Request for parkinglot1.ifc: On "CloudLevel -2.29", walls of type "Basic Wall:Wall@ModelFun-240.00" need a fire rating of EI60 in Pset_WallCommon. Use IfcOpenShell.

First a look at what the model holds.

```python
import ifcopenshell
import ifcopenshell.util.element

model = ifcopenshell.open("parkinglot1.ifc")
print(model.schema)
storey = next(s for s in model.by_type("IfcBuildingStorey") if s.Name == "CloudLevel -2.29")
walls = [e for e in ifcopenshell.util.element.get_decomposition(storey) if e.is_a("IfcWall")]
seen = {}
for e in walls:
    element_type = ifcopenshell.util.element.get_type(e)
    key = (element_type.Name if element_type != e and element_type else None, ifcopenshell.util.element.get_pset(e, "Pset_WallCommon", "FireRating"))
    seen[key] = seen.get(key, 0) + 1
for (name, value), count in sorted(seen.items(), key=str):
    print(count, "x", name, "|", value)
```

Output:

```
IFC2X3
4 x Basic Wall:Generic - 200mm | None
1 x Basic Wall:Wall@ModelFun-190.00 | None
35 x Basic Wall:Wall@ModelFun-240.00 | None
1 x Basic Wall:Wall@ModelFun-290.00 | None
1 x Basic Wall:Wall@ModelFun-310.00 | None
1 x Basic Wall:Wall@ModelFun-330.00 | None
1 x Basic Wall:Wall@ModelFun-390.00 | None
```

```python
import ifcopenshell
import ifcopenshell.api.pset
import ifcopenshell.util.element

model = ifcopenshell.open("parkinglot1.ifc")

storey = next(s for s in model.by_type("IfcBuildingStorey") if s.Name == "CloudLevel -2.29")
walls = [e for e in ifcopenshell.util.element.get_decomposition(storey) if e.is_a("IfcWall")]

count = 0
for e in walls:
    element_type = ifcopenshell.util.element.get_type(e)
    if element_type in (None, e) or element_type.Name != "Basic Wall:Wall@ModelFun-240.00":
        continue
    # add_pset returns the element's existing set when there is one.
    pset = ifcopenshell.api.pset.add_pset(model, product=e, name="Pset_WallCommon")
    ifcopenshell.api.pset.edit_pset(model, pset=pset, properties={"FireRating": "EI60"})
    count += 1

print(count, "walls updated")

model.write("parkinglot1-out.ifc")
```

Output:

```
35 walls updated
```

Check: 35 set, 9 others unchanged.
